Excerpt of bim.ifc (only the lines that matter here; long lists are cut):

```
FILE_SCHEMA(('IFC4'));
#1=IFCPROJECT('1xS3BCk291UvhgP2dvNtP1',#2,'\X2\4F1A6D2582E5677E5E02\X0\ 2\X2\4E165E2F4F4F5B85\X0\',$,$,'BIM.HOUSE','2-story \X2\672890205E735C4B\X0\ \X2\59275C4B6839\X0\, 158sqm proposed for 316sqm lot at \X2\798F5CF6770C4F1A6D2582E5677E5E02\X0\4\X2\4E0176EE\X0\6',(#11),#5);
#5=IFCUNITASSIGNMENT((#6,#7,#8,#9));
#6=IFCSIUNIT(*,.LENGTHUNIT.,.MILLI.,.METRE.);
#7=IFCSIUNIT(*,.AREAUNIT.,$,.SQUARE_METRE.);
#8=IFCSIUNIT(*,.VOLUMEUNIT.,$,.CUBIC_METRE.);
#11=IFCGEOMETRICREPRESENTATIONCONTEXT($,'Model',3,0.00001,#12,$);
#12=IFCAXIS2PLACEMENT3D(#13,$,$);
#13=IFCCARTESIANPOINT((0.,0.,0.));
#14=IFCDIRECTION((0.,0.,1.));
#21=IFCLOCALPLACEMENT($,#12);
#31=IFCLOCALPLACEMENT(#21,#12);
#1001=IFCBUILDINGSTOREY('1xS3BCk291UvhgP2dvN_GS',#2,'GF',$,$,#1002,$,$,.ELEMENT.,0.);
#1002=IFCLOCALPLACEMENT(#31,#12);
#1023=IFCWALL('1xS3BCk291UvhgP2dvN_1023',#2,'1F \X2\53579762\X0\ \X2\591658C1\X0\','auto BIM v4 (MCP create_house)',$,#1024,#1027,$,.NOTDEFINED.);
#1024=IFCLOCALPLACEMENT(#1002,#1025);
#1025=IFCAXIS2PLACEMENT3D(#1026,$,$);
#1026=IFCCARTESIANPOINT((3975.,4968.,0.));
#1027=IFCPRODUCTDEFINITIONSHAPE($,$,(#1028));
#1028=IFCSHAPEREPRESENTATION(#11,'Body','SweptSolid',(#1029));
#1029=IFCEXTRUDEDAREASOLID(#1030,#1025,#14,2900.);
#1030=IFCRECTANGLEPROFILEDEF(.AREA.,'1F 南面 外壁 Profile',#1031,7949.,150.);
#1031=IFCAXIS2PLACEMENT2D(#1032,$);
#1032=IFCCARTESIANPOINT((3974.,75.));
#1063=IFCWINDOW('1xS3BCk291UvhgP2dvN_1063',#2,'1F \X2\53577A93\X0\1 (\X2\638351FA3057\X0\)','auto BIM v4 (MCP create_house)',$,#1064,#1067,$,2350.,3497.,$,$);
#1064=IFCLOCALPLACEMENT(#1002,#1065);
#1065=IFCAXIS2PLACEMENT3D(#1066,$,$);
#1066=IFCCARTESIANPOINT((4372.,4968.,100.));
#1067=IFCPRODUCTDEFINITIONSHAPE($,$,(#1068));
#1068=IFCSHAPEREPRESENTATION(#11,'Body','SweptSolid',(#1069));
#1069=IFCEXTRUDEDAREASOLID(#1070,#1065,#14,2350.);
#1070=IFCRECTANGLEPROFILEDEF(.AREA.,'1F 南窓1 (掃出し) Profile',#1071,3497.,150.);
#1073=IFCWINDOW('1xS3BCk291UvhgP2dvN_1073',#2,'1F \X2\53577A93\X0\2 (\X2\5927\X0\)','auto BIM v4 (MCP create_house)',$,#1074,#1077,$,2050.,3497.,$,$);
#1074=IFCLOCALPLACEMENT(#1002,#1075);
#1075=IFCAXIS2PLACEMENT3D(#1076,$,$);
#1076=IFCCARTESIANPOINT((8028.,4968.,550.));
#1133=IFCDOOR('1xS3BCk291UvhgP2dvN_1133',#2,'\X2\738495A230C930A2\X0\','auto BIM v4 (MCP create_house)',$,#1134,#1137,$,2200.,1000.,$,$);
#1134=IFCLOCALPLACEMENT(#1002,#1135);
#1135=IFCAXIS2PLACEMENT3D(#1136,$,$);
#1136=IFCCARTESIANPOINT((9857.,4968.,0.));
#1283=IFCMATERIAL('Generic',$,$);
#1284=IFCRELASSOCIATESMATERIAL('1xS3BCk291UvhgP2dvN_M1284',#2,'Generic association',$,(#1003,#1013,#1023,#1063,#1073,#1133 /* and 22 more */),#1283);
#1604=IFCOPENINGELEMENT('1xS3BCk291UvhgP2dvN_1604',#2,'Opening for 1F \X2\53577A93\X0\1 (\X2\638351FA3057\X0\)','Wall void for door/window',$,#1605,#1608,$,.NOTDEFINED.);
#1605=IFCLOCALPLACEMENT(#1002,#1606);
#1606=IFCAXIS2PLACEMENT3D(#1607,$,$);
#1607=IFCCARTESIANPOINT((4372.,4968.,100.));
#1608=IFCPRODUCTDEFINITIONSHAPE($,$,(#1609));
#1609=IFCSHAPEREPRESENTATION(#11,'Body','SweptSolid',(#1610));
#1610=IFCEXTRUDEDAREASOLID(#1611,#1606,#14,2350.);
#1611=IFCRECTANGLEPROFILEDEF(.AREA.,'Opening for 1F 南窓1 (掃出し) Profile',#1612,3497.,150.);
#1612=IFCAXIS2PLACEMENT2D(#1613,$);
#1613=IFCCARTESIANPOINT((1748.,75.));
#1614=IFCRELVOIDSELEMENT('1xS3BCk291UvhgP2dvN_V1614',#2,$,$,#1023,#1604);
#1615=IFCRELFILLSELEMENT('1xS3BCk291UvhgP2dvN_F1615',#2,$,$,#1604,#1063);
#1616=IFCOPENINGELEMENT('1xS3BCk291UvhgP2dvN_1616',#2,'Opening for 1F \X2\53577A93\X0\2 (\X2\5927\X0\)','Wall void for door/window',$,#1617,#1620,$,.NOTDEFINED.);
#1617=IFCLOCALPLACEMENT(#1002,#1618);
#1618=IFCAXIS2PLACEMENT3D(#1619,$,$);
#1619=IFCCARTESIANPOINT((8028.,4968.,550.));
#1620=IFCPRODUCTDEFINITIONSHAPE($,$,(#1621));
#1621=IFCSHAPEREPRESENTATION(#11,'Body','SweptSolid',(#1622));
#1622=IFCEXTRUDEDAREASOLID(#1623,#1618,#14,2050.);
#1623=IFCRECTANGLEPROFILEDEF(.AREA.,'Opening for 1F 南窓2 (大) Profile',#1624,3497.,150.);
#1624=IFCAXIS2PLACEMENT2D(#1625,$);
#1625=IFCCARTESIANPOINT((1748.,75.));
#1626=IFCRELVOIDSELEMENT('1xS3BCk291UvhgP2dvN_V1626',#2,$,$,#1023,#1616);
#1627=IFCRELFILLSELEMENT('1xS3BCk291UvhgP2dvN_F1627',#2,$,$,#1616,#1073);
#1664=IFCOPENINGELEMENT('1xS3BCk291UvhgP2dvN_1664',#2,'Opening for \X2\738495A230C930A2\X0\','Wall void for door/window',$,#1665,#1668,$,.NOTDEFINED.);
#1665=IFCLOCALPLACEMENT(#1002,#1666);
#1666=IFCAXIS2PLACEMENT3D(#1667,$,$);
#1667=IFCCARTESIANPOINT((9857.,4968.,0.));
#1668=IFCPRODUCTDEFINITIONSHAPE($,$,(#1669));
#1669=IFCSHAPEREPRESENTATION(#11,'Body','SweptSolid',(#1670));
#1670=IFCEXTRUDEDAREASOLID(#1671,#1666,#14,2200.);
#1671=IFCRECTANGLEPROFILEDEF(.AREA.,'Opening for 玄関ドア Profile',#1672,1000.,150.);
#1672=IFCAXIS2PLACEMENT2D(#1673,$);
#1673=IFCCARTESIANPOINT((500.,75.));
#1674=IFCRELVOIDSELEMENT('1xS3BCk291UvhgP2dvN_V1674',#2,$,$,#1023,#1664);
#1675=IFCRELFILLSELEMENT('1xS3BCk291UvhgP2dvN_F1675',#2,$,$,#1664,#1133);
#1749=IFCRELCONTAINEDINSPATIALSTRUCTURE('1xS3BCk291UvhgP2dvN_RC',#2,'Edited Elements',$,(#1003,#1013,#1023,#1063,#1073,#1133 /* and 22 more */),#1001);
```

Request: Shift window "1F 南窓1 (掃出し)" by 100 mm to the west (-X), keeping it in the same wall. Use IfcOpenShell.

```python
import ifcopenshell
import ifcopenshell.api.geometry
import ifcopenshell.util.placement

model = ifcopenshell.open("bim.ifc")

window = model.by_id(1063)
opening = window.FillsVoids[0].RelatingOpeningElement
wall = opening.VoidsElements[0].RelatingBuildingElement

wall_matrix = ifcopenshell.util.placement.get_local_placement(wall.ObjectPlacement)
shift = wall_matrix[:3, 0] * -100.0
before = ifcopenshell.util.placement.get_local_placement(window.ObjectPlacement)[:3, 3].copy()

# The window is not placed relative to its opening, so move both.
for product in (opening, window):
    matrix = ifcopenshell.util.placement.get_local_placement(product.ObjectPlacement)
    matrix[:3, 3] += shift
    ifcopenshell.api.geometry.edit_object_placement(model, product=product, matrix=matrix, is_si=False)

after = ifcopenshell.util.placement.get_local_placement(window.ObjectPlacement)[:3, 3]
print("window moved by", (after - before).round(3) + 0.0)

model.write("bim_updated.ifc")
```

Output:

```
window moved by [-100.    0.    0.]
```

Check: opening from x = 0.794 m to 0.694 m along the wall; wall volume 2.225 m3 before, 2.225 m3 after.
